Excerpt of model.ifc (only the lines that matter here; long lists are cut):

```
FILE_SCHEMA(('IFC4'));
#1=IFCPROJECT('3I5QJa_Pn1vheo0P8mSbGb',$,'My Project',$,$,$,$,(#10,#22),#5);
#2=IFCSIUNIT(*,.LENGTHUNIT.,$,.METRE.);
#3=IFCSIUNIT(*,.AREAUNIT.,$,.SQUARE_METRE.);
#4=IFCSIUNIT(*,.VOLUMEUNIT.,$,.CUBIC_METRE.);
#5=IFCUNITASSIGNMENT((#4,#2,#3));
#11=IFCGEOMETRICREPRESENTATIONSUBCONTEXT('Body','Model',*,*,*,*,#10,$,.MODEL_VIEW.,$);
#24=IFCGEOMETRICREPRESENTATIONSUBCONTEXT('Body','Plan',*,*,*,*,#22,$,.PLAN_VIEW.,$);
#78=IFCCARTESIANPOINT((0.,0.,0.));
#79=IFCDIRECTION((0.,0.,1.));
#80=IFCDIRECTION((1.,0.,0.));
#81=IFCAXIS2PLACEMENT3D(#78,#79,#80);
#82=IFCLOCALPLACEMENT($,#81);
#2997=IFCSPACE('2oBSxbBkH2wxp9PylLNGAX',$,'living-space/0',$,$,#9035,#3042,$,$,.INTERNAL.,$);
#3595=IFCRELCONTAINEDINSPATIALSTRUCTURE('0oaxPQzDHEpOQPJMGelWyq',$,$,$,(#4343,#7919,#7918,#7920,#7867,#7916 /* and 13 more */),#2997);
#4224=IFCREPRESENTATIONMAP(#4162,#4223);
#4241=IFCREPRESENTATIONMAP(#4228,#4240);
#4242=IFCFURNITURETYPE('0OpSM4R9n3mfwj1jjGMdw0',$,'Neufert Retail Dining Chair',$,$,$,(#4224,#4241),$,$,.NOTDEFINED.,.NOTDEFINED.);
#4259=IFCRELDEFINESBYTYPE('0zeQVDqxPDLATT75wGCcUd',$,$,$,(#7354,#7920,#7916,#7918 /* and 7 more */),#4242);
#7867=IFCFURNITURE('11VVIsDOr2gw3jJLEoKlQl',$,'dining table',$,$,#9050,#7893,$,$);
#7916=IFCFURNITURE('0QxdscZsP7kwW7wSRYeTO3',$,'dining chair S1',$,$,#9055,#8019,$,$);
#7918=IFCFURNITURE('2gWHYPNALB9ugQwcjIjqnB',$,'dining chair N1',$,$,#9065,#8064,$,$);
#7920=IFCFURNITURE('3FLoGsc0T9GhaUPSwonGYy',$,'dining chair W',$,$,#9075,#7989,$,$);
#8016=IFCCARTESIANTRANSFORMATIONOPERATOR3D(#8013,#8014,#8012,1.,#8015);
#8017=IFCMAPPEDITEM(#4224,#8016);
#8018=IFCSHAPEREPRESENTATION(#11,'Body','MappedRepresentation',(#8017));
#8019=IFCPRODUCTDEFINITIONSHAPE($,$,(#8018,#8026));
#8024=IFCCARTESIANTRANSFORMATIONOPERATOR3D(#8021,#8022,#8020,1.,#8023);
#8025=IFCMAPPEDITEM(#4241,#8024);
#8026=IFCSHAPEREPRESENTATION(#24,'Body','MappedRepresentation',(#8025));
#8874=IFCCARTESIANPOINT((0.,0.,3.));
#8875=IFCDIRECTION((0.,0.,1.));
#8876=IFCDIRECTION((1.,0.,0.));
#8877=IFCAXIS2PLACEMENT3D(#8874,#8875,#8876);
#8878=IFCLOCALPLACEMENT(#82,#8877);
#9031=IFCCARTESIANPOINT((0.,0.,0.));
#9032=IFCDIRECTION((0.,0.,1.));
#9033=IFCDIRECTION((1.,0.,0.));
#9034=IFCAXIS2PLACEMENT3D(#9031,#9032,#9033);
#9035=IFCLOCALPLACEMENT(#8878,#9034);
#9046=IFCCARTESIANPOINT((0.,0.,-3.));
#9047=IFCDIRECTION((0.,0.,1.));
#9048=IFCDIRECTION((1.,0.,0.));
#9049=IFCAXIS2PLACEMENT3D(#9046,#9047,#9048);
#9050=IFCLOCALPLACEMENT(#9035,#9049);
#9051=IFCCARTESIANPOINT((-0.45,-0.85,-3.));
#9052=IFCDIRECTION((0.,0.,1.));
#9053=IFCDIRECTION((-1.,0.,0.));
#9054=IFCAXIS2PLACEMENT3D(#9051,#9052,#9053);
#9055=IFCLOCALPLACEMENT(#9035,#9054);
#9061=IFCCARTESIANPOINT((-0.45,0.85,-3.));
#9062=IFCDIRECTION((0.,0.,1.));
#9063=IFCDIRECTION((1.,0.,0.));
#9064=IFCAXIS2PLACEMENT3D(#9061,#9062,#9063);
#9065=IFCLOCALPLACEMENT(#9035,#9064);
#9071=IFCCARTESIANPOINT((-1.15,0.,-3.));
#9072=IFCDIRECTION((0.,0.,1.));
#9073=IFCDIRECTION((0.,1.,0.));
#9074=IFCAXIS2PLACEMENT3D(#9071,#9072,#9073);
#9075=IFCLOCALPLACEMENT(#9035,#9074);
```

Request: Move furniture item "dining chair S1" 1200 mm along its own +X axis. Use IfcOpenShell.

```python
import ifcopenshell
import ifcopenshell.api.geometry
import ifcopenshell.util.placement
import ifcopenshell.util.unit

model = ifcopenshell.open("model.ifc")
unit_scale = ifcopenshell.util.unit.calculate_unit_scale(model)

item = model.by_guid("0QxdscZsP7kwW7wSRYeTO3")
matrix = ifcopenshell.util.placement.get_local_placement(item.ObjectPlacement)
matrix[:3, 3] += matrix[:3, 0] * 1.2 / unit_scale
ifcopenshell.api.geometry.edit_object_placement(model, product=item, matrix=matrix, is_si=False)

print(ifcopenshell.util.placement.get_local_placement(item.ObjectPlacement).round(3) + 0.0)

model.write("model_edited.ifc")
```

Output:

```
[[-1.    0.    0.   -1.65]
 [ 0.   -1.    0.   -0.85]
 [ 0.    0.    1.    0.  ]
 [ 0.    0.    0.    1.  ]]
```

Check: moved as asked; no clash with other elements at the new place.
